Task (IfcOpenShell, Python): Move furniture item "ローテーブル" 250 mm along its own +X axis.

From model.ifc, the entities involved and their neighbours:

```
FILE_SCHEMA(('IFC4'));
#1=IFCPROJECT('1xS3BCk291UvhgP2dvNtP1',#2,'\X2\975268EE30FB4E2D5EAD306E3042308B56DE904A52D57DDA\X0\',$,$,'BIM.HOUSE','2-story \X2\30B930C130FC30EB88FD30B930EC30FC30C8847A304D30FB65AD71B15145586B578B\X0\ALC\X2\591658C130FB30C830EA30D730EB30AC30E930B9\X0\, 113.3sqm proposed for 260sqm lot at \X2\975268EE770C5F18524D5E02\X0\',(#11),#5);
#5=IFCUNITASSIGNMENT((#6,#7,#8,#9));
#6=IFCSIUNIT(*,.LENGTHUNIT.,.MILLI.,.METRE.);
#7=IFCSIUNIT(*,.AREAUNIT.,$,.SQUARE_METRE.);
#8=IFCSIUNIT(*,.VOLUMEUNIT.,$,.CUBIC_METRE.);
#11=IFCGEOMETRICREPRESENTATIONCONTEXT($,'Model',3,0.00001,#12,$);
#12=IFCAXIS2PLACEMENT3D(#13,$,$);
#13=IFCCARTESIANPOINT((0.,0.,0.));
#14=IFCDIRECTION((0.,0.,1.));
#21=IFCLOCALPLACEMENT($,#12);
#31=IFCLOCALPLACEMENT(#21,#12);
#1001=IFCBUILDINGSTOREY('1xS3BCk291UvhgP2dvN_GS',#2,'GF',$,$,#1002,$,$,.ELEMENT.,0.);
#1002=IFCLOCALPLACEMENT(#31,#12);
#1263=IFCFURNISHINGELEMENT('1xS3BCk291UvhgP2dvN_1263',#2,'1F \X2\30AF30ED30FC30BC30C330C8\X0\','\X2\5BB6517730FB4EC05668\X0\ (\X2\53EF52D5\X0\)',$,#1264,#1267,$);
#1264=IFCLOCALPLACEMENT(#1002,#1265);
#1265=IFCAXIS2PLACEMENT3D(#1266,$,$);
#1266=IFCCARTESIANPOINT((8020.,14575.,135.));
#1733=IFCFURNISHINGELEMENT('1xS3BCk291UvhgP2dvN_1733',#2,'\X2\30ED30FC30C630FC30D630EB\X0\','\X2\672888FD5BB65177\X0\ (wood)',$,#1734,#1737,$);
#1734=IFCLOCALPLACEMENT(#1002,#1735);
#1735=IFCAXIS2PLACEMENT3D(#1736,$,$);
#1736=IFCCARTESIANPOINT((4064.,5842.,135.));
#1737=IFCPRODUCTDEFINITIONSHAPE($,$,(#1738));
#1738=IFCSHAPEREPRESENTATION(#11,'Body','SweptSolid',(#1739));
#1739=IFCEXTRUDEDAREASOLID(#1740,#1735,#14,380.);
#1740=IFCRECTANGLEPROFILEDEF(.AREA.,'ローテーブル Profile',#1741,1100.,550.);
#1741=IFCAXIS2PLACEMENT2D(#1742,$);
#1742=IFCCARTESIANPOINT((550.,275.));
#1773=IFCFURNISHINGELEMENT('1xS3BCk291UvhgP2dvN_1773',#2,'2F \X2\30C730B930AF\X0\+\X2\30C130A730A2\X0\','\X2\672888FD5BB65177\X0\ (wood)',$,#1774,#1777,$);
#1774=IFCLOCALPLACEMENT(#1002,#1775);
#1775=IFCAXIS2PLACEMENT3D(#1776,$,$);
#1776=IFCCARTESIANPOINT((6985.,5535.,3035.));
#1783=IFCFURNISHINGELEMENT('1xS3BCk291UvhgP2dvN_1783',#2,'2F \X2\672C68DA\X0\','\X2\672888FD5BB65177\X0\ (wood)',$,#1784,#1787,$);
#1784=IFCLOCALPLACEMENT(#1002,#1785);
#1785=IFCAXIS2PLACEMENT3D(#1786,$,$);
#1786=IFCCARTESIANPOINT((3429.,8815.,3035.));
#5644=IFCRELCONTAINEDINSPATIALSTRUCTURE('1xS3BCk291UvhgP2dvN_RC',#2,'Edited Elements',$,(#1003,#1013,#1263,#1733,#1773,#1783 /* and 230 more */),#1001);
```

```python
import ifcopenshell
import ifcopenshell.api.geometry
import ifcopenshell.util.placement

model = ifcopenshell.open("model.ifc")

item = model.by_guid("1xS3BCk291UvhgP2dvN_1733")
matrix = ifcopenshell.util.placement.get_local_placement(item.ObjectPlacement)
matrix[:3, 3] += matrix[:3, 0] * 250.0
ifcopenshell.api.geometry.edit_object_placement(model, product=item, matrix=matrix, is_si=False)

print(ifcopenshell.util.placement.get_local_placement(item.ObjectPlacement).round(3) + 0.0)

model.write("model_edited.ifc")
```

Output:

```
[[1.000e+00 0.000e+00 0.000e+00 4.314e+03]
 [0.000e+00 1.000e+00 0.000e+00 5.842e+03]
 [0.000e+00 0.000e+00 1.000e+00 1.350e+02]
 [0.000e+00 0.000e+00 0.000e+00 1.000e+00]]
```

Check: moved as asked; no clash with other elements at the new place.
